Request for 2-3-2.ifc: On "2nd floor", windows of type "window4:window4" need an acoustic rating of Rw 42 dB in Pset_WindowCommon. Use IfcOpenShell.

First a look at what the model holds.

```python
import ifcopenshell
import ifcopenshell.util.element

model = ifcopenshell.open("2-3-2.ifc")
print(model.schema)
storey = next(s for s in model.by_type("IfcBuildingStorey") if s.Name == "2nd floor")
windows = [e for e in ifcopenshell.util.element.get_decomposition(storey) if e.is_a("IfcWindow")]
seen = {}
for e in windows:
    element_type = ifcopenshell.util.element.get_type(e)
    key = (element_type.Name if element_type != e and element_type else None, ifcopenshell.util.element.get_pset(e, "Pset_WindowCommon", "AcousticRating"))
    seen[key] = seen.get(key, 0) + 1
for (name, value), count in sorted(seen.items(), key=str):
    print(count, "x", name, "|", value)
```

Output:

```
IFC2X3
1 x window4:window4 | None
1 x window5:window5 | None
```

```python
import ifcopenshell
import ifcopenshell.api.pset
import ifcopenshell.util.element

model = ifcopenshell.open("2-3-2.ifc")

storey = next(s for s in model.by_type("IfcBuildingStorey") if s.Name == "2nd floor")
windows = [e for e in ifcopenshell.util.element.get_decomposition(storey) if e.is_a("IfcWindow")]

count = 0
for e in windows:
    element_type = ifcopenshell.util.element.get_type(e)
    if element_type in (None, e) or element_type.Name != "window4:window4":
        continue
    # add_pset returns the element's existing set when there is one.
    pset = ifcopenshell.api.pset.add_pset(model, product=e, name="Pset_WindowCommon")
    ifcopenshell.api.pset.edit_pset(model, pset=pset, properties={"AcousticRating": "Rw 42 dB"})
    count += 1

print(count, "windows updated")

model.write("2-3-2_updated.ifc")
```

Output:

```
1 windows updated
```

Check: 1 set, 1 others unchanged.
